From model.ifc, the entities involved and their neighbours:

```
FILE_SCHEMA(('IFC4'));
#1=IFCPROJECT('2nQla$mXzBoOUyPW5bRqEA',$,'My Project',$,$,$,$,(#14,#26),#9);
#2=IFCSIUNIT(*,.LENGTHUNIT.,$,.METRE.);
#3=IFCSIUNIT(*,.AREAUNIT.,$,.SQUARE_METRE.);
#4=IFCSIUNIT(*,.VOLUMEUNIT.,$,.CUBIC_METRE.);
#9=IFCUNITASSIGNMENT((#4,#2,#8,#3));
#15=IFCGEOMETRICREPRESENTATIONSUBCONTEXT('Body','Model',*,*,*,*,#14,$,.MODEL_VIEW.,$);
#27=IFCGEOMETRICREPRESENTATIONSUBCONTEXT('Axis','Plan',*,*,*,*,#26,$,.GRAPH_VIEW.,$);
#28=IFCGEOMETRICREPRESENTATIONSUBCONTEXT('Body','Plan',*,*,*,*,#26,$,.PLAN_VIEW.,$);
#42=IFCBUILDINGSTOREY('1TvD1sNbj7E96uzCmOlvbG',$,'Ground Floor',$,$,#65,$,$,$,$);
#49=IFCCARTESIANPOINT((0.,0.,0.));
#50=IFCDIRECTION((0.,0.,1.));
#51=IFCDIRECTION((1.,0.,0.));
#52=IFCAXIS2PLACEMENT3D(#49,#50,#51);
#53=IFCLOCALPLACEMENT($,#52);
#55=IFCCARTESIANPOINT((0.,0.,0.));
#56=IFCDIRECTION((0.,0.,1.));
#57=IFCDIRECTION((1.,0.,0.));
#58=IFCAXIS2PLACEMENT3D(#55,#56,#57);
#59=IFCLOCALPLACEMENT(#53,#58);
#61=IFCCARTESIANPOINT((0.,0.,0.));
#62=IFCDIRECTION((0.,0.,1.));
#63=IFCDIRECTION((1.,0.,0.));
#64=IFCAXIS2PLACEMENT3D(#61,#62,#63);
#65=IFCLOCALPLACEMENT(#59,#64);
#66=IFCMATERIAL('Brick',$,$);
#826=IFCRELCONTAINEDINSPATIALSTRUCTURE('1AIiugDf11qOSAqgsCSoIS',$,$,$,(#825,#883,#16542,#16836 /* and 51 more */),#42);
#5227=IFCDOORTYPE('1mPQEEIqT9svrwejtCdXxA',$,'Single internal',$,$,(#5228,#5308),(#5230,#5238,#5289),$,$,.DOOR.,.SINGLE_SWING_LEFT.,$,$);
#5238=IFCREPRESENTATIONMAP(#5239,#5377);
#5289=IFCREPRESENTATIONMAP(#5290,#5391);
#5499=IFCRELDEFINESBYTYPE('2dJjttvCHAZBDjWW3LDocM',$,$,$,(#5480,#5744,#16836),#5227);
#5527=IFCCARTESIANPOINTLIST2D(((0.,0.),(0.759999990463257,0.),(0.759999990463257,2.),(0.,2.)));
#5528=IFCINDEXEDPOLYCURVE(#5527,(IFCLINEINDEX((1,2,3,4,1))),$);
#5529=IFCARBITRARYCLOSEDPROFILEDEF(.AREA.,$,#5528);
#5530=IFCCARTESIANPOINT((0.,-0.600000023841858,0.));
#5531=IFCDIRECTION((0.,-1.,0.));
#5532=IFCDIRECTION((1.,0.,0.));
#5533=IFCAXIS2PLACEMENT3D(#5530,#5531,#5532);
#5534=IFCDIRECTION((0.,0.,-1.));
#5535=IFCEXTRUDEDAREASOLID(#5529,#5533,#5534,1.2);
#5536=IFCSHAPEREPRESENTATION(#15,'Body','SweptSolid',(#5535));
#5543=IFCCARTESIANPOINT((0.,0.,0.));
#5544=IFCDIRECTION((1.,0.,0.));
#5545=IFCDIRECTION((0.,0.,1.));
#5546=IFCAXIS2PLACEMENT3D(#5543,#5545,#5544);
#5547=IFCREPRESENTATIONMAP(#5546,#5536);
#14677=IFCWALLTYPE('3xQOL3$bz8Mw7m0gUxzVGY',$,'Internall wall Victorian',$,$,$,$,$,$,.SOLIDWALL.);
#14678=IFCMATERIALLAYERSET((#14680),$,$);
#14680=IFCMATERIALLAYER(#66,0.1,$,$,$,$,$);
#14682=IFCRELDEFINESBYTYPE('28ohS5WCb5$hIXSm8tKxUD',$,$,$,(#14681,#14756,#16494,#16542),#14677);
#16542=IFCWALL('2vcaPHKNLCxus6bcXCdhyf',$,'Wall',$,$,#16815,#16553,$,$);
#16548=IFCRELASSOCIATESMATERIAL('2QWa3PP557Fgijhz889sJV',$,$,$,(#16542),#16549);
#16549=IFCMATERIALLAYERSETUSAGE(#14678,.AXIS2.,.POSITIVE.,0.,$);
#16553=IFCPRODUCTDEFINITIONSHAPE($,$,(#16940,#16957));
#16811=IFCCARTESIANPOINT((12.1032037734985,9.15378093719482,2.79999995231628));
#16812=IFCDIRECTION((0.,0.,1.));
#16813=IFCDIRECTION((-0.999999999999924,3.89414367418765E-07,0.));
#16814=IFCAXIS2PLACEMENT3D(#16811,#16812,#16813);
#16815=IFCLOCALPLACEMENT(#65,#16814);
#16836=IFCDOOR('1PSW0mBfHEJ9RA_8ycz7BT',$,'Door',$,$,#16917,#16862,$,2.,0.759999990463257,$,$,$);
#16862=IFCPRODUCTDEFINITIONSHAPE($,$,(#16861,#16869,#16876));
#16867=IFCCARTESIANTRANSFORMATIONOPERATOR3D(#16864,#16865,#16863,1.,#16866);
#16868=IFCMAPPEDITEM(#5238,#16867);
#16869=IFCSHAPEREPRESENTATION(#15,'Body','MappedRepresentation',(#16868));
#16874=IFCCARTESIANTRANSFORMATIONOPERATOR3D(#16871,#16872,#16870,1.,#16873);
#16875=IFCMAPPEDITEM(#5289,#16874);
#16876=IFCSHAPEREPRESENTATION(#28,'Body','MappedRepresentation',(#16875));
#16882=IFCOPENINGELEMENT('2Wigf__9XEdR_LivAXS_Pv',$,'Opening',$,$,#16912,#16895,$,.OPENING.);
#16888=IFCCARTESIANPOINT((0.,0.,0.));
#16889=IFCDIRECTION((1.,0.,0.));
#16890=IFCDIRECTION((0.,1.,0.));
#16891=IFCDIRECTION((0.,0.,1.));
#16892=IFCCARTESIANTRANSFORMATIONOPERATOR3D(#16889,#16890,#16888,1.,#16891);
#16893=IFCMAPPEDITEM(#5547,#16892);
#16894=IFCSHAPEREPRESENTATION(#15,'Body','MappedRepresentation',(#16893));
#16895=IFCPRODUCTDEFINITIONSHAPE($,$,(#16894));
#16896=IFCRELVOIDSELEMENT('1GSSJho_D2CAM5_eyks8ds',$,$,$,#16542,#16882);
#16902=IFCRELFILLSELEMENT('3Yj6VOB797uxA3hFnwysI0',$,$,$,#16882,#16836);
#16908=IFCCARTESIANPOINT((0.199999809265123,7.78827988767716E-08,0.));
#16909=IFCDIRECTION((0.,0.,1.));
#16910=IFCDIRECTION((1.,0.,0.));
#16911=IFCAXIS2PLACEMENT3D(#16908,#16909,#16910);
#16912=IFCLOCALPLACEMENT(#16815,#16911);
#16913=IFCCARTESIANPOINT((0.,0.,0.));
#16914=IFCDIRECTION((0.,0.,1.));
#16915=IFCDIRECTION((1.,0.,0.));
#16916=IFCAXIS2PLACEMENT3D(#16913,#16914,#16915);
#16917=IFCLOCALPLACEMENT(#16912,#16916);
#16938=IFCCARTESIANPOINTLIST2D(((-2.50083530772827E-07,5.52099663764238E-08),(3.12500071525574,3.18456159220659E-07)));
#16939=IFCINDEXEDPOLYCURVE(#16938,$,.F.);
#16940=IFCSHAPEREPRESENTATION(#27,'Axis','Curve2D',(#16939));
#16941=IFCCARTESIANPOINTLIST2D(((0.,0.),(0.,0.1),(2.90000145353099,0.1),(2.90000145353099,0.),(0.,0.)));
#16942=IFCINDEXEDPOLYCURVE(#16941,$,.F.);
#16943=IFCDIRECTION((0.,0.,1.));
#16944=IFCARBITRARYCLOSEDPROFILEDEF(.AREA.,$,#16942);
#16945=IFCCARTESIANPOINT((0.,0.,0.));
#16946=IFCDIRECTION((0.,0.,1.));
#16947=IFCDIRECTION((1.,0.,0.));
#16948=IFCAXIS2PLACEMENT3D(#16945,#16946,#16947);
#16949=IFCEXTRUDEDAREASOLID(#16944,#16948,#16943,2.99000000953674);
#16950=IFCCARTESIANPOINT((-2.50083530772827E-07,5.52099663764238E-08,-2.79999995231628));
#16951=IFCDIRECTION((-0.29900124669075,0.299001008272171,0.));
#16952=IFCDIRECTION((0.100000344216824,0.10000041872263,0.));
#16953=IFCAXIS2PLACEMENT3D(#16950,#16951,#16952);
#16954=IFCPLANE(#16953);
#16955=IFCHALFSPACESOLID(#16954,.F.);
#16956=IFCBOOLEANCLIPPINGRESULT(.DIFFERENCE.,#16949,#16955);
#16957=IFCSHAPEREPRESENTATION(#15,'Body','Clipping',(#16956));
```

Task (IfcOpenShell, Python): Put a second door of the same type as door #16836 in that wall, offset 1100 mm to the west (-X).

```python
import ifcopenshell
import ifcopenshell.api.feature
import ifcopenshell.api.geometry
import ifcopenshell.api.root
import ifcopenshell.geom
import ifcopenshell.util.element
import ifcopenshell.util.placement
import ifcopenshell.util.shape
import ifcopenshell.util.unit

model = ifcopenshell.open("model.ifc")
unit_scale = ifcopenshell.util.unit.calculate_unit_scale(model)
settings = ifcopenshell.geom.settings()


def volume(element):
    """Net volume in cubic metres, openings subtracted."""
    shape = ifcopenshell.geom.create_shape(settings, element)
    return ifcopenshell.util.shape.get_volume(shape.geometry)


door = model.by_id(16836)
opening = door.FillsVoids[0].RelatingOpeningElement
wall = opening.VoidsElements[0].RelatingBuildingElement
before = volume(wall)
shift = ifcopenshell.util.placement.get_local_placement(wall.ObjectPlacement)[:3, 0] * 1.1 / unit_scale

# copy_class copies the void relationship, type, container and properties, but no geometry.
new_opening = ifcopenshell.api.root.copy_class(model, product=opening)
new_opening.Representation = ifcopenshell.util.element.copy_deep(
    model, opening.Representation, exclude=["IfcGeometricRepresentationContext", "IfcRepresentationMap"]
)
new_door = ifcopenshell.api.root.copy_class(model, product=door)
new_door.Representation = ifcopenshell.util.element.copy_deep(
    model, door.Representation, exclude=["IfcGeometricRepresentationContext", "IfcRepresentationMap"]
)
ifcopenshell.api.feature.add_filling(model, opening=new_opening, element=new_door)

for old, new in ((opening, new_opening), (door, new_door)):
    matrix = ifcopenshell.util.placement.get_local_placement(old.ObjectPlacement)
    matrix[:3, 3] += shift
    ifcopenshell.api.geometry.edit_object_placement(model, product=new, matrix=matrix, is_si=False)

after = volume(wall)

print(f"wall volume {before:.3f} -> {after:.3f} m3")

model.write("model_v2.ifc")
```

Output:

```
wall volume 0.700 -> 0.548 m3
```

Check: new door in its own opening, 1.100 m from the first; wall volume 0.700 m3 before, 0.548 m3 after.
